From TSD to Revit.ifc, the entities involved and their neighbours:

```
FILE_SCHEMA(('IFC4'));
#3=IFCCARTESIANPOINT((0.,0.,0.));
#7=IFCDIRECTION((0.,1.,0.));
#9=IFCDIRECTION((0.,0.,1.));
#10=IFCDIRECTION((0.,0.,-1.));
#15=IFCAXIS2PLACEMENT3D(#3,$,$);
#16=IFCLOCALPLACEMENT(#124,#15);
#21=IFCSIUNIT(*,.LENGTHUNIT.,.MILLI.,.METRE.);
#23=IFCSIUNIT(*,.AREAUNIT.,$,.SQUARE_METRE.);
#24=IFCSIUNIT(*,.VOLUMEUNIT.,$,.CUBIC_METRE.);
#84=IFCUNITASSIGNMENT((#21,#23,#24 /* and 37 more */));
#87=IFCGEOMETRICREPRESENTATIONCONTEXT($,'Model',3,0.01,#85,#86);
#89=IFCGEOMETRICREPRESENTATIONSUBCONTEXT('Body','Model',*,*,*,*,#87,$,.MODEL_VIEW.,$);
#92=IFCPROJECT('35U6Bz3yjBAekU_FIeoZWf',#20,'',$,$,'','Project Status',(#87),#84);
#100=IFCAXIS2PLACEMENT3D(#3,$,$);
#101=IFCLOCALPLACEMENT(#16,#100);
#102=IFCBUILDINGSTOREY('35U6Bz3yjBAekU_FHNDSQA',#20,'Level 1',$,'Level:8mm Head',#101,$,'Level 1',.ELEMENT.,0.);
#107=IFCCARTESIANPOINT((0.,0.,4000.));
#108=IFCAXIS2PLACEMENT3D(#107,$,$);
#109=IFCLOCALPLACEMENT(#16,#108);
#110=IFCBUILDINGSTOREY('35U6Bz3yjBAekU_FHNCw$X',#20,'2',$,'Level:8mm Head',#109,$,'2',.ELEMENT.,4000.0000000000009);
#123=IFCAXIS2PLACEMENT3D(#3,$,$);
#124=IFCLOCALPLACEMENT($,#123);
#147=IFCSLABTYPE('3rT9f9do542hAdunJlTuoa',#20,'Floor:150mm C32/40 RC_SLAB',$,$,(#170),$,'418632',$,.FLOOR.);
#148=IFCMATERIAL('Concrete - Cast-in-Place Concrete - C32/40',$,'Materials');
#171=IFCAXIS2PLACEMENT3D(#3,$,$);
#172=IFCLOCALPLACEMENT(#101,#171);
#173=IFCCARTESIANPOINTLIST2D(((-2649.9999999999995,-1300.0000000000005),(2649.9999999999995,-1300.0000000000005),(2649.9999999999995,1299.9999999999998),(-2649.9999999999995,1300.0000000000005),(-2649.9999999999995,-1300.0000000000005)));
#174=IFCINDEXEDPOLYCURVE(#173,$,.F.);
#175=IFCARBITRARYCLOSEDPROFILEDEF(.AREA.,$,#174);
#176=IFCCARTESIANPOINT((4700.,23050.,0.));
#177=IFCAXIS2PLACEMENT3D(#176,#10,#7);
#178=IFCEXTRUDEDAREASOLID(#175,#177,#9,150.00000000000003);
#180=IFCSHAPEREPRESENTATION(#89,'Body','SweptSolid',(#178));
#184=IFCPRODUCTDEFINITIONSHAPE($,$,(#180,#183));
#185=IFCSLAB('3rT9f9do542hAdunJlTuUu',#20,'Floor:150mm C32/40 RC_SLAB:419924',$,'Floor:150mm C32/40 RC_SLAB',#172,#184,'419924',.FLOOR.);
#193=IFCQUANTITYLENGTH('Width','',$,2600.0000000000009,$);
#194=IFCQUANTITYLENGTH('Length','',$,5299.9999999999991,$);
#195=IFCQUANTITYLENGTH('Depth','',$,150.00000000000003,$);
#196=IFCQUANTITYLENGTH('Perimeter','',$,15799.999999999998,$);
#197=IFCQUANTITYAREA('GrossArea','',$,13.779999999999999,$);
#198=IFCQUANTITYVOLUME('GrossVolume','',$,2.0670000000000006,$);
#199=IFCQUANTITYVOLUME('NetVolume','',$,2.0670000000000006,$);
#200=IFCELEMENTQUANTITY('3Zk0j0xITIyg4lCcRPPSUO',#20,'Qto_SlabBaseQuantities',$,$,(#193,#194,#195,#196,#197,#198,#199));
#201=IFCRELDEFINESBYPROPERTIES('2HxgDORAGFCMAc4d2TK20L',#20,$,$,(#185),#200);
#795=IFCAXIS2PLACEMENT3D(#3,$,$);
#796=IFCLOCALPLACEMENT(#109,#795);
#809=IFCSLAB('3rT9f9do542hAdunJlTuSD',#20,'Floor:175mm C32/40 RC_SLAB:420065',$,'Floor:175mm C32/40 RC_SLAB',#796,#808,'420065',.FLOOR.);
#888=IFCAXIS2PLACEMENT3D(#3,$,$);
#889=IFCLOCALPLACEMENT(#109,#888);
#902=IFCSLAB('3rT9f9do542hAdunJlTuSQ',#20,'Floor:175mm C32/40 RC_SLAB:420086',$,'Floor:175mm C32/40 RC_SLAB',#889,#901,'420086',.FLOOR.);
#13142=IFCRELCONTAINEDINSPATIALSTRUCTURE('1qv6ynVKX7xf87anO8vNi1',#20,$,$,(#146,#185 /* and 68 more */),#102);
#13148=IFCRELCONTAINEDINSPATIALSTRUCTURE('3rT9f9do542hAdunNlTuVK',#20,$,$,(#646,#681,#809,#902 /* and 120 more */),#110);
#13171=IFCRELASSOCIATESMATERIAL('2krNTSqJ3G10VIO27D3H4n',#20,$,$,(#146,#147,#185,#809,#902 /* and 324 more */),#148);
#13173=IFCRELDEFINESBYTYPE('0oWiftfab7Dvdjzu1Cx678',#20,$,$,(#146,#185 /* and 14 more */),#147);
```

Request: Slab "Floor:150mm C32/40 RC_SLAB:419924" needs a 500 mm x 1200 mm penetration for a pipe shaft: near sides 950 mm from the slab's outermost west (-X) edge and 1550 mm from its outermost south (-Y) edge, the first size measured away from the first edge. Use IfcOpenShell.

```python
import numpy as np
import ifcopenshell
import ifcopenshell.api.feature
import ifcopenshell.api.geometry
import ifcopenshell.api.pset
import ifcopenshell.api.root
import ifcopenshell.geom
import ifcopenshell.util.element
import ifcopenshell.util.placement
import ifcopenshell.util.representation
import ifcopenshell.util.shape
import ifcopenshell.util.unit

model = ifcopenshell.open("TSD to Revit.ifc")
unit_scale = ifcopenshell.util.unit.calculate_unit_scale(model)
volume_scale = ifcopenshell.util.unit.calculate_unit_scale(model, "VOLUMEUNIT")
settings = ifcopenshell.geom.settings()


def volume(element):
    """Net volume in cubic metres, openings subtracted."""
    shape = ifcopenshell.geom.create_shape(settings, element)
    return ifcopenshell.util.shape.get_volume(shape.geometry)


slab = model.by_guid("3rT9f9do542hAdunJlTuUu")
before = volume(slab)

# Extent in the slab's own axes, in metres. The edges named are its -X and -Y sides.
slab_shape = ifcopenshell.geom.create_shape(settings, slab)
vertices = ifcopenshell.util.shape.get_vertices(slab_shape.geometry)
x_min, y_min, bottom = vertices.min(axis=0)
top = vertices[:, 2].max()

opening = ifcopenshell.api.root.create_entity(model, ifc_class="IfcOpeningElement", name="Pipe shaft opening", predefined_type="OPENING")
context = ifcopenshell.util.representation.get_context(model, "Model", "Body", "MODEL_VIEW")
width, depth = 0.5, 1.2
outline = [(0.0, 0.0), (width, 0.0), (width, depth), (0.0, depth), (0.0, 0.0)]
# Overshoot both faces by 50 mm so the cut is clean.
shape = ifcopenshell.api.geometry.add_slab_representation(
    model, context=context, depth=top - bottom + 0.1, polyline=outline
)
ifcopenshell.api.geometry.assign_representation(model, product=opening, representation=shape)

matrix = ifcopenshell.util.placement.get_local_placement(slab.ObjectPlacement)
matrix[:, 3] = matrix @ np.append(np.array([x_min + 0.95, y_min + 1.55, bottom - 0.05]) / unit_scale, 1.0)
ifcopenshell.api.geometry.edit_object_placement(model, product=opening, matrix=matrix, is_si=False)
ifcopenshell.api.feature.add_feature(model, feature=opening, element=slab)

after = volume(slab)

# Update the slab's stored quantities.
qto = model.by_id(ifcopenshell.util.element.get_pset(slab, "Qto_SlabBaseQuantities", should_inherit=False)["id"])
ifcopenshell.api.pset.edit_qto(model, qto=qto, properties={"NetVolume": after / volume_scale})

print(f"slab volume {before:.3f} -> {after:.3f} m3")

model.write("TSD to Revit_updated.ifc")
```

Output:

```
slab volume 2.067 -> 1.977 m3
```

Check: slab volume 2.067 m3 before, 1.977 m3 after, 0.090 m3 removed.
